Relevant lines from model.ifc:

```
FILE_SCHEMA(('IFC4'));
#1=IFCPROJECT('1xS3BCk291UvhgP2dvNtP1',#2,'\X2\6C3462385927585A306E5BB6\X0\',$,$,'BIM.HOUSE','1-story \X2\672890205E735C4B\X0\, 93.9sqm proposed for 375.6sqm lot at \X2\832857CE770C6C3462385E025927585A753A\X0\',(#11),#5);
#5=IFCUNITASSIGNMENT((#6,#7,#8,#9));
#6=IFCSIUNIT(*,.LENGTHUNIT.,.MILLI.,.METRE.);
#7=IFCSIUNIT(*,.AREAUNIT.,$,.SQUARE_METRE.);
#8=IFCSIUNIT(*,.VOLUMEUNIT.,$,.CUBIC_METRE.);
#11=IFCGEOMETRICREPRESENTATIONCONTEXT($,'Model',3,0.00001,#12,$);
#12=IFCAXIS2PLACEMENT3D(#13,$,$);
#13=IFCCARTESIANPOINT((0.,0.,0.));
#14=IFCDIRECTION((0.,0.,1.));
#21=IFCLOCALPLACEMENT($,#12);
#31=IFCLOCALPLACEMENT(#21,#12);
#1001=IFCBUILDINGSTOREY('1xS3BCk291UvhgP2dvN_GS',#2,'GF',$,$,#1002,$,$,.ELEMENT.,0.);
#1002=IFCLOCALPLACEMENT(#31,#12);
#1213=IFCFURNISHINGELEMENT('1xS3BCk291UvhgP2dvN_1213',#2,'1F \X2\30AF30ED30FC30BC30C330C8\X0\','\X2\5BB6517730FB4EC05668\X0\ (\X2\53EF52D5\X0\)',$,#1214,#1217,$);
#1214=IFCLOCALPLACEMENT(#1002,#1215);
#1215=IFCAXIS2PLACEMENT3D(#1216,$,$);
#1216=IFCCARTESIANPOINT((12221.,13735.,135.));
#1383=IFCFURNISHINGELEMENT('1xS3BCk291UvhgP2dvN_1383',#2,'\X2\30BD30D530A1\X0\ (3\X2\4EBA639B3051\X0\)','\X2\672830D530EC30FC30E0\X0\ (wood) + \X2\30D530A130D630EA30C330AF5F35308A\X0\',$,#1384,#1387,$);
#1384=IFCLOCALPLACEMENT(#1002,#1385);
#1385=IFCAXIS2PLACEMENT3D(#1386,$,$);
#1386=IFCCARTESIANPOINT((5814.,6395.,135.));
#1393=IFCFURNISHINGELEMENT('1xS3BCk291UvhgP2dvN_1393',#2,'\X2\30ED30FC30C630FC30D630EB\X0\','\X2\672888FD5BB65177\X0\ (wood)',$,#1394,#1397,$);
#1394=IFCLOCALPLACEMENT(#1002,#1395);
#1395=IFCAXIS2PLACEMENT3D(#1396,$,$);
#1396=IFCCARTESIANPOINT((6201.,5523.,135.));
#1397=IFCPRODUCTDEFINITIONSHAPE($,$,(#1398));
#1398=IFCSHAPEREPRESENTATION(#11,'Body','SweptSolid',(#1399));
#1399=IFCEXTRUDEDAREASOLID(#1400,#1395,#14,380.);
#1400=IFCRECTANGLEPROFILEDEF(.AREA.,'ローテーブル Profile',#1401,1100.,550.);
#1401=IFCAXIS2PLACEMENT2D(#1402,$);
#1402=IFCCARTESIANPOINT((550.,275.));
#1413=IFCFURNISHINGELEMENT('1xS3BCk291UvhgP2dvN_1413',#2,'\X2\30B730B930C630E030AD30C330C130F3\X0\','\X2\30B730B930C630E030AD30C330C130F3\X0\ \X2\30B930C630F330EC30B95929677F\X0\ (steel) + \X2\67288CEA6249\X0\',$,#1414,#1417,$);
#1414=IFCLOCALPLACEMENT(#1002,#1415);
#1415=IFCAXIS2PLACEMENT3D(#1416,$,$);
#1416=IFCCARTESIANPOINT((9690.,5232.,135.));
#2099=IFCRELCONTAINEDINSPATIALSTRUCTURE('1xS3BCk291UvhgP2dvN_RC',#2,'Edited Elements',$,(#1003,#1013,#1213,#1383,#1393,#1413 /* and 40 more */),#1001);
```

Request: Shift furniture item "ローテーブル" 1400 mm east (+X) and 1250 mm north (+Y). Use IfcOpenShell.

```python
import ifcopenshell
import ifcopenshell.api.geometry
import ifcopenshell.util.placement

model = ifcopenshell.open("model.ifc")

item = model.by_guid("1xS3BCk291UvhgP2dvN_1393")
matrix = ifcopenshell.util.placement.get_local_placement(item.ObjectPlacement)
matrix[0, 3] += 1400.0
matrix[1, 3] += 1250.0
ifcopenshell.api.geometry.edit_object_placement(model, product=item, matrix=matrix, is_si=False)

print(ifcopenshell.util.placement.get_local_placement(item.ObjectPlacement).round(3) + 0.0)

model.write("model_v2.ifc")
```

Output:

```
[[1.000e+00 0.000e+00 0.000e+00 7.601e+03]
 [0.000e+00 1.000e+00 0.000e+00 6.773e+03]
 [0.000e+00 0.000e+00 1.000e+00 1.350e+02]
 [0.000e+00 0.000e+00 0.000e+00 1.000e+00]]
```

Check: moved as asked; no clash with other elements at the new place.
